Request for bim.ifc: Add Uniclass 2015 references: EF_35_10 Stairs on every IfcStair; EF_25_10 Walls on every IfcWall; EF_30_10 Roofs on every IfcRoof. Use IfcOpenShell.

First a look at what the model holds.

```python
import ifcopenshell

model = ifcopenshell.open("bim.ifc")
print(model.schema)
print("classifications:", [c.Name for c in model.by_type("IfcClassification")])
for ifc_class in ("IfcDoor", "IfcRoof", "IfcStair", "IfcWall", "IfcWindow"):
    print(ifc_class, len(model.by_type(ifc_class)))
```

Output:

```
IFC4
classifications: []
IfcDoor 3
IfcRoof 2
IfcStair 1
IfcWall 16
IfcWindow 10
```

```python
import ifcopenshell
import ifcopenshell.api.classification

model = ifcopenshell.open("bim.ifc")

system = ifcopenshell.api.classification.add_classification(model, classification="Uniclass 2015")

codes = {
    "IfcStair": ("EF_35_10", "Stairs"),
    "IfcWall": ("EF_25_10", "Walls"),
    "IfcRoof": ("EF_30_10", "Roofs"),
}
for ifc_class, (code, name) in codes.items():
    products = model.by_type(ifc_class)
    ifcopenshell.api.classification.add_reference(
        model, products=products, classification=system, identification=code, name=name
    )
    print(code, len(products))

model.write("bim_updated.ifc")
```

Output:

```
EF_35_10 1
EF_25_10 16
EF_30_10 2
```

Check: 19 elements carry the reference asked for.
